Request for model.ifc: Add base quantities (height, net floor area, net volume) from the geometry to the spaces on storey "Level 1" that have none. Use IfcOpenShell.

First a look at what the model holds.

```python
import ifcopenshell
import ifcopenshell.util.element
import ifcopenshell.util.unit

model = ifcopenshell.open("model.ifc")
print(model.schema)
for unit_type in ("LENGTHUNIT", "AREAUNIT", "VOLUMEUNIT"):
    print(unit_type, ifcopenshell.util.unit.calculate_unit_scale(model, unit_type))
storey = next(s for s in model.by_type("IfcBuildingStorey") if s.Name == "Level 1")
spaces = [e for e in ifcopenshell.util.element.get_decomposition(storey) if e.is_a("IfcSpace")]
for e in sorted(spaces, key=lambda e: e.id()):
    print(e.id(), e.is_a(), e.Name, list(ifcopenshell.util.element.get_psets(e, qtos_only=True)), sep=" | ")
```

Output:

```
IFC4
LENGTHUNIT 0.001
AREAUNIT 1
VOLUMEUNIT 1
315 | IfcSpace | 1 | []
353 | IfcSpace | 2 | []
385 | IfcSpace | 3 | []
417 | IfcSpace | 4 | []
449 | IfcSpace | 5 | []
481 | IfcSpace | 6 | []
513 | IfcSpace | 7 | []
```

```python
import ifcopenshell
import ifcopenshell.api.pset
import ifcopenshell.geom
import ifcopenshell.util.element
import ifcopenshell.util.shape
import ifcopenshell.util.unit

model = ifcopenshell.open("model.ifc")
unit_scale = ifcopenshell.util.unit.calculate_unit_scale(model)
area_scale = ifcopenshell.util.unit.calculate_unit_scale(model, "AREAUNIT")
volume_scale = ifcopenshell.util.unit.calculate_unit_scale(model, "VOLUMEUNIT")
settings = ifcopenshell.geom.settings()

storey = next(s for s in model.by_type("IfcBuildingStorey") if s.Name == "Level 1")
spaces = [e for e in ifcopenshell.util.element.get_decomposition(storey) if e.is_a("IfcSpace")]

for e in sorted(spaces, key=lambda e: e.id()):
    if ifcopenshell.util.element.get_psets(e, qtos_only=True, should_inherit=False):
        continue
    # Geometry comes back in metres, in the element's own axes.
    shape = ifcopenshell.geom.create_shape(settings, e)
    values = {
        "Height": ifcopenshell.util.shape.get_z(shape.geometry) / unit_scale,
        "NetFloorArea": ifcopenshell.util.shape.get_footprint_area(shape.geometry) / area_scale,
        "NetVolume": ifcopenshell.util.shape.get_volume(shape.geometry) / volume_scale,
    }
    qto = ifcopenshell.api.pset.add_qto(model, product=e, name="Qto_SpaceBaseQuantities")
    ifcopenshell.api.pset.edit_qto(model, qto=qto, properties=values)
    print(e.id(), {k: round(v, 3) for k, v in values.items()})

model.write("model_v2.ifc")
```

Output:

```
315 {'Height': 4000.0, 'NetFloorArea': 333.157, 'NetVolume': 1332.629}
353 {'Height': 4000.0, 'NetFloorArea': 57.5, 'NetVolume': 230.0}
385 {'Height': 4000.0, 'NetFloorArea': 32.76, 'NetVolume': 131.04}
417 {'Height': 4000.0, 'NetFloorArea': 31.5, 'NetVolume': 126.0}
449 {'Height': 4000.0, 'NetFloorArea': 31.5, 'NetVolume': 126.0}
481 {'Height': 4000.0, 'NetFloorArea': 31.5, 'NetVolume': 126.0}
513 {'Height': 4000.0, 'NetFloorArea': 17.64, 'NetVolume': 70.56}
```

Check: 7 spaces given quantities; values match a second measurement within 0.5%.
